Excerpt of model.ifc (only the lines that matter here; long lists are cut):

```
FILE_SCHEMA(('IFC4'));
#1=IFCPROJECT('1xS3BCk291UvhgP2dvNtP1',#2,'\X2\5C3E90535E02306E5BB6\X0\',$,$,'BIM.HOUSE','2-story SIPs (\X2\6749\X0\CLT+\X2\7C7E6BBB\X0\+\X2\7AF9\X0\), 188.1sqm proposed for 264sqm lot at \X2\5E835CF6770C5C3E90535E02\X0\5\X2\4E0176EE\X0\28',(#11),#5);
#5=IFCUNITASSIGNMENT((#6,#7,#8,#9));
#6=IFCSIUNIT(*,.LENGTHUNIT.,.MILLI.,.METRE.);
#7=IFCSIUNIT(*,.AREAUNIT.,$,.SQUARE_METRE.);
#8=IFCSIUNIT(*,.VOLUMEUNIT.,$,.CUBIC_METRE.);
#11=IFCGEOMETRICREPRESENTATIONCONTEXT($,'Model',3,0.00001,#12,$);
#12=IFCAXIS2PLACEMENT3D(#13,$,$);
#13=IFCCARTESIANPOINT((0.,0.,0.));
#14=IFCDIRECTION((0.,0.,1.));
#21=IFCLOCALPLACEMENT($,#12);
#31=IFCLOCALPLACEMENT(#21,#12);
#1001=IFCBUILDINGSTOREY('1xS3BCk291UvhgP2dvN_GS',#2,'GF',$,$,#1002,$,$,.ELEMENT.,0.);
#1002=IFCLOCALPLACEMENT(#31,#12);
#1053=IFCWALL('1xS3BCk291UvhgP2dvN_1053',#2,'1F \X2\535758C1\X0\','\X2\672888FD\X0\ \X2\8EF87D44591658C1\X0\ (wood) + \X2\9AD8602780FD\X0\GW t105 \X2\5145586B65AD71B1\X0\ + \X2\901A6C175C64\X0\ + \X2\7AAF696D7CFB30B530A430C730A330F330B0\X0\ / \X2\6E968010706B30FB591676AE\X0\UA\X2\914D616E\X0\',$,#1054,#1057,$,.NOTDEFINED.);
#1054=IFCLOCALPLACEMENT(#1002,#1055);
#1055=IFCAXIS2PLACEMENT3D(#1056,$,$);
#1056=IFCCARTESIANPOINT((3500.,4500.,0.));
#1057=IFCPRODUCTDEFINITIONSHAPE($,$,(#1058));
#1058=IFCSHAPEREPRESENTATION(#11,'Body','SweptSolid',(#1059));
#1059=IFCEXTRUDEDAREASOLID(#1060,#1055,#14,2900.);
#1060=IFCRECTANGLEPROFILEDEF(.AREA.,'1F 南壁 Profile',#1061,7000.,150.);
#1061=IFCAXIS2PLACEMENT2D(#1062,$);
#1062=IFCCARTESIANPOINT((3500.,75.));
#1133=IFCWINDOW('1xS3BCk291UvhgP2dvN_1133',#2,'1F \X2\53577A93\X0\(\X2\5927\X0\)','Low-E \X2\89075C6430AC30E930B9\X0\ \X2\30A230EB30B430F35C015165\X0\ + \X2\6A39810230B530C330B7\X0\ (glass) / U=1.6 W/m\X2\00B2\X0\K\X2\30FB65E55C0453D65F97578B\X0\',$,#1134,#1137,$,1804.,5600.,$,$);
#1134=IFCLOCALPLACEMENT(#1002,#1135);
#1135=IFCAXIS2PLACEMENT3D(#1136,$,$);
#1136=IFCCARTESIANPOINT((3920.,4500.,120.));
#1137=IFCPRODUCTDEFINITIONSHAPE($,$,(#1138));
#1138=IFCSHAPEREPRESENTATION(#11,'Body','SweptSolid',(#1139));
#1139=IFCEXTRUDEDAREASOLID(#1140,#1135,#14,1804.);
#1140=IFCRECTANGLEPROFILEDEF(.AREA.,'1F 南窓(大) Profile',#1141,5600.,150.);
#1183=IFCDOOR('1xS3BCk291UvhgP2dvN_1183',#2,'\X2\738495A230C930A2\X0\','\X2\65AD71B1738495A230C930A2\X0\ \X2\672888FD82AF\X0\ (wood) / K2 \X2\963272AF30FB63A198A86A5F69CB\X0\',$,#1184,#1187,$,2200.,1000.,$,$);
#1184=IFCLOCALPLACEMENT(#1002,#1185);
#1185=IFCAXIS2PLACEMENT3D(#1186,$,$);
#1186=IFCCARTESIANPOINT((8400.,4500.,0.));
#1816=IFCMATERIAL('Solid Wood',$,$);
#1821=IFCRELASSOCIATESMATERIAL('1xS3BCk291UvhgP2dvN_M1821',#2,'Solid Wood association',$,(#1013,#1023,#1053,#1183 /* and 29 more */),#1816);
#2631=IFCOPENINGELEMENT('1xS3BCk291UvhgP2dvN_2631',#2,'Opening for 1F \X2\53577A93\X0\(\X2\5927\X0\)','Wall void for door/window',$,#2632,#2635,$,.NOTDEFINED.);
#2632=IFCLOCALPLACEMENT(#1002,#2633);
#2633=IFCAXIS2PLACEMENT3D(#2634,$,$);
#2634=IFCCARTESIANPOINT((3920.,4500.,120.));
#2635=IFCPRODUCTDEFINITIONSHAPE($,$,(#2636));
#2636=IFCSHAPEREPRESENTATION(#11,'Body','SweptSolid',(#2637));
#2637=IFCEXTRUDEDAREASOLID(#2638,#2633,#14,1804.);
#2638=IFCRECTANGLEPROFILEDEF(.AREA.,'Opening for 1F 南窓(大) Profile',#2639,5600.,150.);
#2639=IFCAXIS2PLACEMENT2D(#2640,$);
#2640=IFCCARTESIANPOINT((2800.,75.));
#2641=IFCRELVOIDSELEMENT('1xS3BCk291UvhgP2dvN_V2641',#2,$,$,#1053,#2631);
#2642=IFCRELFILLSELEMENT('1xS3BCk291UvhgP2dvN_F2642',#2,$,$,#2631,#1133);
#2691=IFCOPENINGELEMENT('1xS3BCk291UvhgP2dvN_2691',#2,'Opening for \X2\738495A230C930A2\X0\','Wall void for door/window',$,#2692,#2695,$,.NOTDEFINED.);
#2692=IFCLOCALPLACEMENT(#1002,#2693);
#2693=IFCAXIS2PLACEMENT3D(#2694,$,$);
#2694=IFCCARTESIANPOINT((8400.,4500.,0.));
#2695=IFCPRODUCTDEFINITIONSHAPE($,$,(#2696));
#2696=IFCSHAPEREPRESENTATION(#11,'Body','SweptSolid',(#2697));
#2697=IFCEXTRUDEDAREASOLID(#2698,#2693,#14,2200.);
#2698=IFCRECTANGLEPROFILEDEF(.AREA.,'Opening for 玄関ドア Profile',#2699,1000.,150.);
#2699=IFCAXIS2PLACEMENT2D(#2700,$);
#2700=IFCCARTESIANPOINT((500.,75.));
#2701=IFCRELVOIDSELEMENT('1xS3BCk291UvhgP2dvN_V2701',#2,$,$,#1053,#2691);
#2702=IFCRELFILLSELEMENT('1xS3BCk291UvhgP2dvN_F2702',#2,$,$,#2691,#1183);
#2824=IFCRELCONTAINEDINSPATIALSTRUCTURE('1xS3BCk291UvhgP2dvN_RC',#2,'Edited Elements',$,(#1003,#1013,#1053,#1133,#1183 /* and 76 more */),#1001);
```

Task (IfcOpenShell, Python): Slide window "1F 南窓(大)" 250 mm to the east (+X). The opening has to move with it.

```python
import ifcopenshell
import ifcopenshell.api.geometry
import ifcopenshell.util.placement
import ifcopenshell.util.unit

model = ifcopenshell.open("model.ifc")
unit_scale = ifcopenshell.util.unit.calculate_unit_scale(model)

window = model.by_id(1133)
opening = window.FillsVoids[0].RelatingOpeningElement
wall = opening.VoidsElements[0].RelatingBuildingElement

wall_matrix = ifcopenshell.util.placement.get_local_placement(wall.ObjectPlacement)
shift = wall_matrix[:3, 0] * 0.25 / unit_scale
before = ifcopenshell.util.placement.get_local_placement(window.ObjectPlacement)[:3, 3].copy()

# The window is not placed relative to its opening, so move both.
for product in (opening, window):
    matrix = ifcopenshell.util.placement.get_local_placement(product.ObjectPlacement)
    matrix[:3, 3] += shift
    ifcopenshell.api.geometry.edit_object_placement(model, product=product, matrix=matrix, is_si=False)

after = ifcopenshell.util.placement.get_local_placement(window.ObjectPlacement)[:3, 3]
print("window moved by", (after - before).round(3) + 0.0)

model.write("model_updated.ifc")
```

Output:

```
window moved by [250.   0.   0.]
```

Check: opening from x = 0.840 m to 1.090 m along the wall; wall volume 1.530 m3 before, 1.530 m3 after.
